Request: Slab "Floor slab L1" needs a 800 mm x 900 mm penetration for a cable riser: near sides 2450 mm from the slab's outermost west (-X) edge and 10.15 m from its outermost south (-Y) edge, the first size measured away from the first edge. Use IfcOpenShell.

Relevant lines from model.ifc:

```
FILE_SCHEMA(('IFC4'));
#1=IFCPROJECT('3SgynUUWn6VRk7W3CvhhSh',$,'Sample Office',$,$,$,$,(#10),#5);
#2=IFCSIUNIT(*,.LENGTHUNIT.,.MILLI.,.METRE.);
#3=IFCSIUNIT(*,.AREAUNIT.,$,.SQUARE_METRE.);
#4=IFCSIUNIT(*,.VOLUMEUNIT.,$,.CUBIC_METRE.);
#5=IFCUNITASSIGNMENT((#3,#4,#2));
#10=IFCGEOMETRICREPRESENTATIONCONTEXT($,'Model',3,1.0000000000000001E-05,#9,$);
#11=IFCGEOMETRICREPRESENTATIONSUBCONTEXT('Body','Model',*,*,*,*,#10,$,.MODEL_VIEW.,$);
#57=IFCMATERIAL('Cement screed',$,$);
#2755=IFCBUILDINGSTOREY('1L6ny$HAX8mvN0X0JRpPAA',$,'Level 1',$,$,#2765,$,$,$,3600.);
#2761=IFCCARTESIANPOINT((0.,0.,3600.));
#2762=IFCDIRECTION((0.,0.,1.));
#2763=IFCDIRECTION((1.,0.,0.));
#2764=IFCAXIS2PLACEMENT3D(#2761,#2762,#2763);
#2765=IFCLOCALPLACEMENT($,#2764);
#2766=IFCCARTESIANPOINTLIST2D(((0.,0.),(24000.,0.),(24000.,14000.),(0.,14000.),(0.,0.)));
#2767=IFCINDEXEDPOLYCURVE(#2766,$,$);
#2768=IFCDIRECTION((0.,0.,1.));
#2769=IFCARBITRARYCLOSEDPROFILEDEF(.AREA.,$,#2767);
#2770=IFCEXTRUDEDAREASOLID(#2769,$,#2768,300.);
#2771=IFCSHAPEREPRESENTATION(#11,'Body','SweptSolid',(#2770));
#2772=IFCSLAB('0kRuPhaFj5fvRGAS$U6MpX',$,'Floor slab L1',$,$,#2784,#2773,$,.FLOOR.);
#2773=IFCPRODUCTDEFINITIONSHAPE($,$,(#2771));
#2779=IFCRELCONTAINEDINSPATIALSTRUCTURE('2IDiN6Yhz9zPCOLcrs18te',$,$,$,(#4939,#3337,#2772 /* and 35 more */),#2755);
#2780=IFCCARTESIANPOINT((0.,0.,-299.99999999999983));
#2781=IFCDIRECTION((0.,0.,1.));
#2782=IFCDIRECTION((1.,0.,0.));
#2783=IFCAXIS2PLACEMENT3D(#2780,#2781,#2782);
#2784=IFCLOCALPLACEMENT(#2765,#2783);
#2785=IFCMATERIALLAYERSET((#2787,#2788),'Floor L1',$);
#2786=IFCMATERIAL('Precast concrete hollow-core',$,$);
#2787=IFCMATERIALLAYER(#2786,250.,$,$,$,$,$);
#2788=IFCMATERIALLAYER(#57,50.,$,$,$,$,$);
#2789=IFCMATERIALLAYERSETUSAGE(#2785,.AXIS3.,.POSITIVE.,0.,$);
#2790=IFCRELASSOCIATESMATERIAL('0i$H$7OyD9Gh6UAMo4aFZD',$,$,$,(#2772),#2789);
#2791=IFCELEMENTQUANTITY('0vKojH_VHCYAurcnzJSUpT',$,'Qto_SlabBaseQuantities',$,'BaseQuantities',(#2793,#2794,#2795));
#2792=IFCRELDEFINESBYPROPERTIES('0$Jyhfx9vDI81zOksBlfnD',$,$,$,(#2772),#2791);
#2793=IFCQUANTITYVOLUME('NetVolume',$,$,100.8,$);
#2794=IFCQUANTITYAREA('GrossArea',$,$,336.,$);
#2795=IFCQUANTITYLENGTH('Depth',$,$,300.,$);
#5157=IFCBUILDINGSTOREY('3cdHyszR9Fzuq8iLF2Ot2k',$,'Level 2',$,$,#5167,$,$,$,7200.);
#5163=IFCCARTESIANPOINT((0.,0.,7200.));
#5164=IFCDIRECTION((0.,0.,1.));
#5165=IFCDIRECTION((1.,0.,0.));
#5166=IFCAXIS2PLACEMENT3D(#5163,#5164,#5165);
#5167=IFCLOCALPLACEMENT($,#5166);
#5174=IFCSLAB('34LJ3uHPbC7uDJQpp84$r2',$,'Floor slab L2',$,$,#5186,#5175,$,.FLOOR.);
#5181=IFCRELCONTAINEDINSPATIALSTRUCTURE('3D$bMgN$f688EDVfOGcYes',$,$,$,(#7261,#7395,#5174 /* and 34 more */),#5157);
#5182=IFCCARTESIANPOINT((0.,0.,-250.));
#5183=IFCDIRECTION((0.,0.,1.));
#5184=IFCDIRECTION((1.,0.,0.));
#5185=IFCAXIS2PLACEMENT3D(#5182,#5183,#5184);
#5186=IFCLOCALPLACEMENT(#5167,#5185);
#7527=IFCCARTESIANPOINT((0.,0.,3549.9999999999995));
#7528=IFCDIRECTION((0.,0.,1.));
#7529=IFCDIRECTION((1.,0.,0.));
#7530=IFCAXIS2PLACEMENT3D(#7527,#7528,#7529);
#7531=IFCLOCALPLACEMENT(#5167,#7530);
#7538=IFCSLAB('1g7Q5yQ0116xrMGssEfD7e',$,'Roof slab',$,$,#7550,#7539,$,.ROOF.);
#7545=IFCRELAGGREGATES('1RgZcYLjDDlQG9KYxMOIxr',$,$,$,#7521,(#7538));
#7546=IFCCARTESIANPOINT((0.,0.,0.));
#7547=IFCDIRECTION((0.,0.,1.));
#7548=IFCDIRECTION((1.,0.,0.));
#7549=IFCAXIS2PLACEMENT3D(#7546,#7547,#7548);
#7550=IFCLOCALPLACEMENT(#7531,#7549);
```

```python
import numpy as np
import ifcopenshell
import ifcopenshell.api.feature
import ifcopenshell.api.geometry
import ifcopenshell.api.pset
import ifcopenshell.api.root
import ifcopenshell.geom
import ifcopenshell.util.element
import ifcopenshell.util.placement
import ifcopenshell.util.representation
import ifcopenshell.util.shape
import ifcopenshell.util.unit

model = ifcopenshell.open("model.ifc")
unit_scale = ifcopenshell.util.unit.calculate_unit_scale(model)
volume_scale = ifcopenshell.util.unit.calculate_unit_scale(model, "VOLUMEUNIT")
settings = ifcopenshell.geom.settings()


def volume(element):
    """Net volume in cubic metres, openings subtracted."""
    shape = ifcopenshell.geom.create_shape(settings, element)
    return ifcopenshell.util.shape.get_volume(shape.geometry)


slab = model.by_guid("0kRuPhaFj5fvRGAS$U6MpX")
before = volume(slab)

# Extent in the slab's own axes, in metres. The edges named are its -X and -Y sides.
slab_shape = ifcopenshell.geom.create_shape(settings, slab)
vertices = ifcopenshell.util.shape.get_vertices(slab_shape.geometry)
x_min, y_min, bottom = vertices.min(axis=0)
top = vertices[:, 2].max()

opening = ifcopenshell.api.root.create_entity(model, ifc_class="IfcOpeningElement", name="Cable riser opening", predefined_type="OPENING")
context = ifcopenshell.util.representation.get_context(model, "Model", "Body", "MODEL_VIEW")
width, depth = 0.8, 0.9
outline = [(0.0, 0.0), (width, 0.0), (width, depth), (0.0, depth), (0.0, 0.0)]
# Overshoot both faces by 50 mm so the cut is clean.
shape = ifcopenshell.api.geometry.add_slab_representation(
    model, context=context, depth=top - bottom + 0.1, polyline=outline
)
ifcopenshell.api.geometry.assign_representation(model, product=opening, representation=shape)

matrix = ifcopenshell.util.placement.get_local_placement(slab.ObjectPlacement)
matrix[:, 3] = matrix @ np.append(np.array([x_min + 2.45, y_min + 10.15, bottom - 0.05]) / unit_scale, 1.0)
ifcopenshell.api.geometry.edit_object_placement(model, product=opening, matrix=matrix, is_si=False)
ifcopenshell.api.feature.add_feature(model, feature=opening, element=slab)

after = volume(slab)

# Update the slab's stored quantities.
qto = model.by_id(ifcopenshell.util.element.get_pset(slab, "Qto_SlabBaseQuantities", should_inherit=False)["id"])
ifcopenshell.api.pset.edit_qto(model, qto=qto, properties={"NetVolume": after / volume_scale})

print(f"slab volume {before:.3f} -> {after:.3f} m3")

model.write("model_edited.ifc")
```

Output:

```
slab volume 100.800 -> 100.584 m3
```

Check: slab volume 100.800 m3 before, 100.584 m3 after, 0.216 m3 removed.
